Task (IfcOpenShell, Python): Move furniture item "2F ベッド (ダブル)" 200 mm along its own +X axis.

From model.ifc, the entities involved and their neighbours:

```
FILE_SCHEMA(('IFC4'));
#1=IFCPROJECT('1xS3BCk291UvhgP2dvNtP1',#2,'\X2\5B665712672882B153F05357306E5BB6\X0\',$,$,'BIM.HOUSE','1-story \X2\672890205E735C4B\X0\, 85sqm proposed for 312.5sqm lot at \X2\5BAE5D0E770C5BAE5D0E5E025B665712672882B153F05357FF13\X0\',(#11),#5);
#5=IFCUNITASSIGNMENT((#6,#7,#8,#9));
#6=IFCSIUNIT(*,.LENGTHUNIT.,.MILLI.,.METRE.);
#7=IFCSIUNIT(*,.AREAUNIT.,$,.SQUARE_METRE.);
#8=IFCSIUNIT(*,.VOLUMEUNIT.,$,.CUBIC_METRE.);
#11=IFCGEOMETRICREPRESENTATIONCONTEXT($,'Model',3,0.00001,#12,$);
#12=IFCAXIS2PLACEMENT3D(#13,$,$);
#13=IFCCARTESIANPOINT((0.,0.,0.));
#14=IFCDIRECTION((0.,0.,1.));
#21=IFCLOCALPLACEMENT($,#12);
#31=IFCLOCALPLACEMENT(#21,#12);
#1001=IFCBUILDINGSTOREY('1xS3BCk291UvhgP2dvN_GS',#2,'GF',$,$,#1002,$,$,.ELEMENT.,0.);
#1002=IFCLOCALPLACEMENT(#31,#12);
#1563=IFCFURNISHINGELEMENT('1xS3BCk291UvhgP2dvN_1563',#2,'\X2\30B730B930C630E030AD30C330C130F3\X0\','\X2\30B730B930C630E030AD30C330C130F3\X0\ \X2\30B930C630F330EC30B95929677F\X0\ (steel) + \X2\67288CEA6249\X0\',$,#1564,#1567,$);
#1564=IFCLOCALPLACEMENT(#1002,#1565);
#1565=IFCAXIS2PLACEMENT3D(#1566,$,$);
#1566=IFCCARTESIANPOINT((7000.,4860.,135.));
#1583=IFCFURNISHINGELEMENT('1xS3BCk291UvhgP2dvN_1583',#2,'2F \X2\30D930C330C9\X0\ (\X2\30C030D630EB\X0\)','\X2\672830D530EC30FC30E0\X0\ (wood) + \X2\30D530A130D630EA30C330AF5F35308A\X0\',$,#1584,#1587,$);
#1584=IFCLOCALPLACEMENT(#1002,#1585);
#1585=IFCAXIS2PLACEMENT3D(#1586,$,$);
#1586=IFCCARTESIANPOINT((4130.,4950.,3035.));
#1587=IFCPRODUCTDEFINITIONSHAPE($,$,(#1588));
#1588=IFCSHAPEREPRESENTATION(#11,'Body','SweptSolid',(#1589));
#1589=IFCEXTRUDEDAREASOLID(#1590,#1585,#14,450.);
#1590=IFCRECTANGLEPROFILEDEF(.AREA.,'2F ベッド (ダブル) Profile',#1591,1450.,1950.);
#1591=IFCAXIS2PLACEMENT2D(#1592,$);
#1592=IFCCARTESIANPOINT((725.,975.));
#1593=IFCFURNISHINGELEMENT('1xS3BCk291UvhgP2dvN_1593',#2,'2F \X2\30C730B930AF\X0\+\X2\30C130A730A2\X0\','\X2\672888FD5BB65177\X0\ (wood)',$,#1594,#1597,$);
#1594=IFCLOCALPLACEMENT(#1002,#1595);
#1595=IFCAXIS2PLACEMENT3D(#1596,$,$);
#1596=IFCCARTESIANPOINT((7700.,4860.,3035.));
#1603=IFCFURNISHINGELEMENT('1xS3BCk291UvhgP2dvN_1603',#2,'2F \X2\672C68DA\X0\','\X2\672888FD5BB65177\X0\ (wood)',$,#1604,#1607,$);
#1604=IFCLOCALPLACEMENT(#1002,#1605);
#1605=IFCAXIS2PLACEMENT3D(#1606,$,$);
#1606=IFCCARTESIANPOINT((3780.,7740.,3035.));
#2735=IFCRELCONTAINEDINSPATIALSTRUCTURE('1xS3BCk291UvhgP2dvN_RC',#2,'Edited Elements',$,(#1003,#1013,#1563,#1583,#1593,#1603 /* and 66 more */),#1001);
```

```python
import ifcopenshell
import ifcopenshell.api.geometry
import ifcopenshell.util.placement
import ifcopenshell.util.unit

model = ifcopenshell.open("model.ifc")
unit_scale = ifcopenshell.util.unit.calculate_unit_scale(model)

item = model.by_guid("1xS3BCk291UvhgP2dvN_1583")
matrix = ifcopenshell.util.placement.get_local_placement(item.ObjectPlacement)
matrix[:3, 3] += matrix[:3, 0] * 0.2 / unit_scale
ifcopenshell.api.geometry.edit_object_placement(model, product=item, matrix=matrix, is_si=False)

print(ifcopenshell.util.placement.get_local_placement(item.ObjectPlacement).round(3) + 0.0)

model.write("model_rev.ifc")
```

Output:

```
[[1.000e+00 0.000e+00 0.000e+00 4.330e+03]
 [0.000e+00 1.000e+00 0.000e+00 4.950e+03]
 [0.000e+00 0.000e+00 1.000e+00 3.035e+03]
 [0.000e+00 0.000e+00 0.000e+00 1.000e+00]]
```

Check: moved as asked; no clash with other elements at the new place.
